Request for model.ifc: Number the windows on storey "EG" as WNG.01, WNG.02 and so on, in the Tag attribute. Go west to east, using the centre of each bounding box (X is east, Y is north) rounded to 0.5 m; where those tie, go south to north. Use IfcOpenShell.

First a look at what the model holds.

```python
import ifcopenshell
import ifcopenshell.util.element
import ifcopenshell.util.placement

model = ifcopenshell.open("model.ifc")
print(model.schema)
storey = next(s for s in model.by_type("IfcBuildingStorey") if s.Name == "EG")
windows = [e for e in ifcopenshell.util.element.get_decomposition(storey) if e.is_a("IfcWindow")]
for e in sorted(windows, key=lambda e: e.id()):
    origin = ifcopenshell.util.placement.get_local_placement(e.ObjectPlacement)[:3, 3]
    print(e.id(), e.Tag, e.Name, origin.round(2) + 0.0, sep=" | ")
```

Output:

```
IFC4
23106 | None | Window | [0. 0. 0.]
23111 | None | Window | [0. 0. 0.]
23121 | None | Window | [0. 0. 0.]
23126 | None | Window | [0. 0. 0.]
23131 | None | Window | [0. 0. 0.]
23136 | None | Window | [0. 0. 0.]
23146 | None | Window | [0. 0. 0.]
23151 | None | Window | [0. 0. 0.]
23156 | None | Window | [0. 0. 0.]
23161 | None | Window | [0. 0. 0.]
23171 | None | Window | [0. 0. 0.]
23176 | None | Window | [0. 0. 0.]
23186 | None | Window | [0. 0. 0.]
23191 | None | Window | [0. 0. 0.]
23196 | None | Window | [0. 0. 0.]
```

```python
import ifcopenshell
import ifcopenshell.geom
import ifcopenshell.util.element
import ifcopenshell.util.shape

model = ifcopenshell.open("model.ifc")
settings = ifcopenshell.geom.settings()
settings.set("use-world-coords", True)


def centre(element):
    shape = ifcopenshell.geom.create_shape(settings, element)
    return ifcopenshell.util.shape.get_bbox_centroid(shape.geometry)


storey = next(s for s in model.by_type("IfcBuildingStorey") if s.Name == "EG")
windows = [e for e in ifcopenshell.util.element.get_decomposition(storey) if e.is_a("IfcWindow")]

# Insertion points can sit at a corner or the storey origin, so sort by the geometry (in metres).
centres = {e: centre(e) for e in windows}
windows.sort(key=lambda e: (round(centres[e][0] / 0.5), centres[e][1]))

for i, e in enumerate(windows, start=1):
    number = f"WNG.{i:02d}"
    e.Tag = number
    print(e.id(), number)

model.write("model-out.ifc")
```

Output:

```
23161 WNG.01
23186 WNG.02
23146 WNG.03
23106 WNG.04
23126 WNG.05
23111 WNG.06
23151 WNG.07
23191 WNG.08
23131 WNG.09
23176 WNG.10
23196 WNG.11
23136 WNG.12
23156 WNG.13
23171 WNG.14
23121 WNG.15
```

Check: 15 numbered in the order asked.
